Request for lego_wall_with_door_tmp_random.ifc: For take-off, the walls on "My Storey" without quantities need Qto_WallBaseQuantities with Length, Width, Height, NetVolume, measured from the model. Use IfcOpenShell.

First a look at what the model holds.

```python
import ifcopenshell
import ifcopenshell.util.element
import ifcopenshell.util.unit

model = ifcopenshell.open("lego_wall_with_door_tmp_random.ifc")
print(model.schema)
for unit_type in ("LENGTHUNIT", "AREAUNIT", "VOLUMEUNIT"):
    print(unit_type, ifcopenshell.util.unit.calculate_unit_scale(model, unit_type))
storey = next(s for s in model.by_type("IfcBuildingStorey") if s.Name == "My Storey")
walls = [e for e in ifcopenshell.util.element.get_decomposition(storey) if e.is_a("IfcWall")]
for e in sorted(walls, key=lambda e: e.id()):
    print(e.id(), e.is_a(), e.Name, list(ifcopenshell.util.element.get_psets(e, qtos_only=True)), sep=" | ")
```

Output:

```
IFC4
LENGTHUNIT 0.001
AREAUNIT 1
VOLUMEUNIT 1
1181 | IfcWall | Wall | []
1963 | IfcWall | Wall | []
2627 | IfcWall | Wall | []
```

```python
import ifcopenshell
import ifcopenshell.api.pset
import ifcopenshell.geom
import ifcopenshell.util.element
import ifcopenshell.util.shape
import ifcopenshell.util.unit

model = ifcopenshell.open("lego_wall_with_door_tmp_random.ifc")
unit_scale = ifcopenshell.util.unit.calculate_unit_scale(model)
volume_scale = ifcopenshell.util.unit.calculate_unit_scale(model, "VOLUMEUNIT")
settings = ifcopenshell.geom.settings()

storey = next(s for s in model.by_type("IfcBuildingStorey") if s.Name == "My Storey")
walls = [e for e in ifcopenshell.util.element.get_decomposition(storey) if e.is_a("IfcWall")]

for e in sorted(walls, key=lambda e: e.id()):
    if ifcopenshell.util.element.get_psets(e, qtos_only=True, should_inherit=False):
        continue
    # Geometry comes back in metres, in the element's own axes.
    shape = ifcopenshell.geom.create_shape(settings, e)
    values = {
        "Length": ifcopenshell.util.shape.get_x(shape.geometry) / unit_scale,
        "Width": ifcopenshell.util.shape.get_y(shape.geometry) / unit_scale,
        "Height": ifcopenshell.util.shape.get_z(shape.geometry) / unit_scale,
        "NetVolume": ifcopenshell.util.shape.get_volume(shape.geometry) / volume_scale,
    }
    qto = ifcopenshell.api.pset.add_qto(model, product=e, name="Qto_WallBaseQuantities")
    ifcopenshell.api.pset.edit_qto(model, qto=qto, properties=values)
    print(e.id(), {k: round(v, 3) for k, v in values.items()})

model.write("lego_wall_with_door_tmp_random_rev.ifc")
```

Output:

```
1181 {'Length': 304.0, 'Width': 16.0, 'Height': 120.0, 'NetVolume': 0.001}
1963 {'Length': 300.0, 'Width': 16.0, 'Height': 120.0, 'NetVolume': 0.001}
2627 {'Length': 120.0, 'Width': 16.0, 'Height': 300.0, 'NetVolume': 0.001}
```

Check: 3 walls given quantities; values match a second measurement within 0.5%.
